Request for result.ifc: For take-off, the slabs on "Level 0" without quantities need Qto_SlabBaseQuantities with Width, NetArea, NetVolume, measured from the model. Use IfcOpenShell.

First a look at what the model holds.

```python
import ifcopenshell
import ifcopenshell.util.element
import ifcopenshell.util.unit

model = ifcopenshell.open("result.ifc")
print(model.schema)
for unit_type in ("LENGTHUNIT", "AREAUNIT", "VOLUMEUNIT"):
    print(unit_type, ifcopenshell.util.unit.calculate_unit_scale(model, unit_type))
storey = next(s for s in model.by_type("IfcBuildingStorey") if s.Name == "Level 0")
slabs = [e for e in ifcopenshell.util.element.get_decomposition(storey) if e.is_a("IfcSlab")]
for e in sorted(slabs, key=lambda e: e.id()):
    print(e.id(), e.is_a(), e.Name, list(ifcopenshell.util.element.get_psets(e, qtos_only=True)), sep=" | ")
```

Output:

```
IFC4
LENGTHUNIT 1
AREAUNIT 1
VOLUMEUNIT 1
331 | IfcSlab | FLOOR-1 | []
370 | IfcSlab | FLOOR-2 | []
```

```python
import ifcopenshell
import ifcopenshell.api.pset
import ifcopenshell.geom
import ifcopenshell.util.element
import ifcopenshell.util.shape
import ifcopenshell.util.unit

model = ifcopenshell.open("result.ifc")
unit_scale = ifcopenshell.util.unit.calculate_unit_scale(model)
area_scale = ifcopenshell.util.unit.calculate_unit_scale(model, "AREAUNIT")
volume_scale = ifcopenshell.util.unit.calculate_unit_scale(model, "VOLUMEUNIT")
settings = ifcopenshell.geom.settings()

storey = next(s for s in model.by_type("IfcBuildingStorey") if s.Name == "Level 0")
slabs = [e for e in ifcopenshell.util.element.get_decomposition(storey) if e.is_a("IfcSlab")]

for e in sorted(slabs, key=lambda e: e.id()):
    if ifcopenshell.util.element.get_psets(e, qtos_only=True, should_inherit=False):
        continue
    # Geometry comes back in metres, in the element's own axes.
    shape = ifcopenshell.geom.create_shape(settings, e)
    values = {
        "Width": ifcopenshell.util.shape.get_z(shape.geometry) / unit_scale,
        "NetArea": ifcopenshell.util.shape.get_footprint_area(shape.geometry) / area_scale,
        "NetVolume": ifcopenshell.util.shape.get_volume(shape.geometry) / volume_scale,
    }
    qto = ifcopenshell.api.pset.add_qto(model, product=e, name="Qto_SlabBaseQuantities")
    ifcopenshell.api.pset.edit_qto(model, qto=qto, properties=values)
    print(e.id(), {k: round(v, 3) for k, v in values.items()})

model.write("result-out.ifc")
```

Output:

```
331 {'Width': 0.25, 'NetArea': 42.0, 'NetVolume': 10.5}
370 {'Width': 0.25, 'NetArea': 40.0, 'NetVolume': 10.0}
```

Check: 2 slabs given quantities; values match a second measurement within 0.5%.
